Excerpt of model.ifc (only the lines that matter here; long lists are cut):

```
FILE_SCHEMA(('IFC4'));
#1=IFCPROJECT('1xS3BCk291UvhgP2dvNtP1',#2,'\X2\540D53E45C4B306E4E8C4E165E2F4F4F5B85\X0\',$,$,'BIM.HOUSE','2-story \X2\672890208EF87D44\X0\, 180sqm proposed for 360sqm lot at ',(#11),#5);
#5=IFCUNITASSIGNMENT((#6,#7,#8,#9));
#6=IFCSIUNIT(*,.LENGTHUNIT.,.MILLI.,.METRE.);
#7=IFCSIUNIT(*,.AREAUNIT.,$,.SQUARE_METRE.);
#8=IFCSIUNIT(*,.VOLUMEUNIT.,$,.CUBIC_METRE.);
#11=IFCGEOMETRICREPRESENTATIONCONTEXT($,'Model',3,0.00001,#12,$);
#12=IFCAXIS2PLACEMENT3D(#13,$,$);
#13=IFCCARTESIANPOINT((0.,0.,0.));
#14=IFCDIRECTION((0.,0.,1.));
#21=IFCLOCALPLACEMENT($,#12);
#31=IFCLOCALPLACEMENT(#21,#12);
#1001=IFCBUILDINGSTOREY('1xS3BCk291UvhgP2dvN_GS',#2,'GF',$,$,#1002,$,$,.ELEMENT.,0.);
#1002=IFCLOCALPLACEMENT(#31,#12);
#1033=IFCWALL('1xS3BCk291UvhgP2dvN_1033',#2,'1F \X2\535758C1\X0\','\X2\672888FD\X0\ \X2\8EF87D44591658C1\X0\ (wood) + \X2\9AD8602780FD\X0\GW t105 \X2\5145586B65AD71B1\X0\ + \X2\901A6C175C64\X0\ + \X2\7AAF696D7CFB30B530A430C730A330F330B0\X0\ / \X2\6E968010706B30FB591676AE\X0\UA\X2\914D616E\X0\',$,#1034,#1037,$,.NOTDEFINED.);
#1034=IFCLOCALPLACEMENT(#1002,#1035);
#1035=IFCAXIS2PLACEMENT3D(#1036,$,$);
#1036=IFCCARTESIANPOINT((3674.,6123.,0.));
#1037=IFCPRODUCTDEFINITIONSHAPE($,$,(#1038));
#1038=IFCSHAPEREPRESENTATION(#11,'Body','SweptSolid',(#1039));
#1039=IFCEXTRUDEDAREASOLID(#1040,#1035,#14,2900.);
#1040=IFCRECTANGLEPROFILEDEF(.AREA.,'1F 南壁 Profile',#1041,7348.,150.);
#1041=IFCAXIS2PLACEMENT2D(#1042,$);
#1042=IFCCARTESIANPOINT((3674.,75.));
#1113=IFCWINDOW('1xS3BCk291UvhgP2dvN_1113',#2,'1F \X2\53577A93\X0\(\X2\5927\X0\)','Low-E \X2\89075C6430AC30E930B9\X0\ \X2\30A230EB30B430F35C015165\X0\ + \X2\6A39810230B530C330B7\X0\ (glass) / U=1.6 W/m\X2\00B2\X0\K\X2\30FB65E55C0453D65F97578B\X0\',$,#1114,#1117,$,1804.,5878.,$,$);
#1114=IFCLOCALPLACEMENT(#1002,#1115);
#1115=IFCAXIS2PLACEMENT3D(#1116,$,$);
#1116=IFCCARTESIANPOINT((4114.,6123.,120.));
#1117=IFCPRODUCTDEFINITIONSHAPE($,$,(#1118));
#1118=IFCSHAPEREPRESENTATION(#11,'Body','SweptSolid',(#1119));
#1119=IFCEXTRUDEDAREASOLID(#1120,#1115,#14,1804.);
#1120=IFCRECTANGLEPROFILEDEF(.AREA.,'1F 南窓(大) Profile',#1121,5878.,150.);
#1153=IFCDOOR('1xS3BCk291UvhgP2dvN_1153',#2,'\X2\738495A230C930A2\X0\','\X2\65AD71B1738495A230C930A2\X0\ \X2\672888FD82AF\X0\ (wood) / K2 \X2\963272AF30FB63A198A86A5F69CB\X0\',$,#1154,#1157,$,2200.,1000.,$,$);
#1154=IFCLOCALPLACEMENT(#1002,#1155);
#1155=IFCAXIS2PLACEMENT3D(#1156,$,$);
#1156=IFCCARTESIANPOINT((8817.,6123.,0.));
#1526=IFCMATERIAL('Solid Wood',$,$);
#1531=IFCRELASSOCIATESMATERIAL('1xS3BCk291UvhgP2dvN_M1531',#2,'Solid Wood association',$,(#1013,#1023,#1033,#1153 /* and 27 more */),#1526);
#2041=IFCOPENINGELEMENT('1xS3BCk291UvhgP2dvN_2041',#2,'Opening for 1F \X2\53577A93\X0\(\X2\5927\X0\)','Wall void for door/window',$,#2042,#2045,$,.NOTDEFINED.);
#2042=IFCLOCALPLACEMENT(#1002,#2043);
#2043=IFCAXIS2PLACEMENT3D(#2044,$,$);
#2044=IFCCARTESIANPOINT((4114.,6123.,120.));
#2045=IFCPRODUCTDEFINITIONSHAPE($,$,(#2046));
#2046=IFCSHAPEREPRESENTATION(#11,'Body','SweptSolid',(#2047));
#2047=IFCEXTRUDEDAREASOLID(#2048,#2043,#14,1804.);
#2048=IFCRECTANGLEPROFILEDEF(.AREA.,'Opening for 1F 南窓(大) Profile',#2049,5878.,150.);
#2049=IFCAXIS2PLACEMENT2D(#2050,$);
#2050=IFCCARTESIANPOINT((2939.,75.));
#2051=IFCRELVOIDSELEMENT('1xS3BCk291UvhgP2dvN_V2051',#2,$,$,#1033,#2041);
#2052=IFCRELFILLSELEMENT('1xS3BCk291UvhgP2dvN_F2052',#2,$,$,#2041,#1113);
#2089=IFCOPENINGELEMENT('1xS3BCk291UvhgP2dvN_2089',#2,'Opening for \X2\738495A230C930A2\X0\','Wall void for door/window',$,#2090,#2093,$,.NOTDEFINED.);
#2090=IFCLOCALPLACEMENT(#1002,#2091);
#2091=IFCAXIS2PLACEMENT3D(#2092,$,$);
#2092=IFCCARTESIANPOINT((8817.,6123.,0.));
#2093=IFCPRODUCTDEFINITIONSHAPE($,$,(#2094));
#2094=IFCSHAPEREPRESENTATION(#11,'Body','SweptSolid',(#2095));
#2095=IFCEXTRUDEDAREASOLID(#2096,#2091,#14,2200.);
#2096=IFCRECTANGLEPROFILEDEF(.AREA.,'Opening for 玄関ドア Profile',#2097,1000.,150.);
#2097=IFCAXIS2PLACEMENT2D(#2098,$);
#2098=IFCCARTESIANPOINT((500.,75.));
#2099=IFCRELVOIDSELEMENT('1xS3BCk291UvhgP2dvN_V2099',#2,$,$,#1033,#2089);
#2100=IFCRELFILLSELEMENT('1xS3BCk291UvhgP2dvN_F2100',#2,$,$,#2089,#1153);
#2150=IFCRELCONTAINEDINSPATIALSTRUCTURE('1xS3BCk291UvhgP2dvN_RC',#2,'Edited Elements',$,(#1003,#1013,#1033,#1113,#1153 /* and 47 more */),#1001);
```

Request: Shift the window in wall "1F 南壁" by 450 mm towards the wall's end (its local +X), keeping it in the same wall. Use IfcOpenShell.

```python
import ifcopenshell
import ifcopenshell.api.geometry
import ifcopenshell.util.placement

model = ifcopenshell.open("model.ifc")

window = model.by_id(1113)
opening = window.FillsVoids[0].RelatingOpeningElement
wall = opening.VoidsElements[0].RelatingBuildingElement

wall_matrix = ifcopenshell.util.placement.get_local_placement(wall.ObjectPlacement)
shift = wall_matrix[:3, 0] * 450.0
before = ifcopenshell.util.placement.get_local_placement(window.ObjectPlacement)[:3, 3].copy()

# The window is not placed relative to its opening, so move both.
for product in (opening, window):
    matrix = ifcopenshell.util.placement.get_local_placement(product.ObjectPlacement)
    matrix[:3, 3] += shift
    ifcopenshell.api.geometry.edit_object_placement(model, product=product, matrix=matrix, is_si=False)

after = ifcopenshell.util.placement.get_local_placement(window.ObjectPlacement)[:3, 3]
print("window moved by", (after - before).round(3) + 0.0)

model.write("model_v2.ifc")
```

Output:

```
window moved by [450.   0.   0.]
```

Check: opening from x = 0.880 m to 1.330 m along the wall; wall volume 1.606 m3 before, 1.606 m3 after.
